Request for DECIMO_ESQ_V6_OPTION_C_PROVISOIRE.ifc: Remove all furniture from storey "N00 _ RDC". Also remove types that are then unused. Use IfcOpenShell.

First a look at what the model holds.

```python
import ifcopenshell
import ifcopenshell.util.element

model = ifcopenshell.open("DECIMO_ESQ_V6_OPTION_C_PROVISOIRE.ifc")
print(model.schema)
storey = next(s for s in model.by_type("IfcBuildingStorey") if s.Name == "N00 _ RDC")
furniture = [e for e in ifcopenshell.util.element.get_decomposition(storey) if e.is_a("IfcFurnishingElement")]
seen = {}
for e in furniture:
    element_type = ifcopenshell.util.element.get_type(e)
    name = element_type.Name if element_type not in (None, e) else None
    seen[name] = seen.get(name, 0) + 1
for name, count in sorted(seen.items(), key=str):
    print(count, "x", name)
```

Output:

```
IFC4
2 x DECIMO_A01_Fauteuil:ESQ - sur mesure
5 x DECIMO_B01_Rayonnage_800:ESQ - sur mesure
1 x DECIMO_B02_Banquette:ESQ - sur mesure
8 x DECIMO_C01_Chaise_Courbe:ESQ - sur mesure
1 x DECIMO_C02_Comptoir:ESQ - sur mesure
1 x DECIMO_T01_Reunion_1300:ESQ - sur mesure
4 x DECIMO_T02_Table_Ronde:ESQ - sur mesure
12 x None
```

```python
import ifcopenshell
import ifcopenshell.api.root
import ifcopenshell.util.element

model = ifcopenshell.open("DECIMO_ESQ_V6_OPTION_C_PROVISOIRE.ifc")

storey = next(s for s in model.by_type("IfcBuildingStorey") if s.Name == "N00 _ RDC")
furniture = [e for e in ifcopenshell.util.element.get_decomposition(storey) if e.is_a("IfcFurnishingElement")]
types = {ifcopenshell.util.element.get_type(e) for e in furniture} - {None, *furniture}

for e in furniture:
    ifcopenshell.api.root.remove_product(model, product=e)
print(len(furniture), "removed")

unused = [t for t in types if not ifcopenshell.util.element.get_types(t)]
for t in unused:
    ifcopenshell.api.root.remove_product(model, product=t)
print(len(unused), "unused types removed")

model.write("DECIMO_ESQ_V6_OPTION_C_PROVISOIRE_v2.ifc")
```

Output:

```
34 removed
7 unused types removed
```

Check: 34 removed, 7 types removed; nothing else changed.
